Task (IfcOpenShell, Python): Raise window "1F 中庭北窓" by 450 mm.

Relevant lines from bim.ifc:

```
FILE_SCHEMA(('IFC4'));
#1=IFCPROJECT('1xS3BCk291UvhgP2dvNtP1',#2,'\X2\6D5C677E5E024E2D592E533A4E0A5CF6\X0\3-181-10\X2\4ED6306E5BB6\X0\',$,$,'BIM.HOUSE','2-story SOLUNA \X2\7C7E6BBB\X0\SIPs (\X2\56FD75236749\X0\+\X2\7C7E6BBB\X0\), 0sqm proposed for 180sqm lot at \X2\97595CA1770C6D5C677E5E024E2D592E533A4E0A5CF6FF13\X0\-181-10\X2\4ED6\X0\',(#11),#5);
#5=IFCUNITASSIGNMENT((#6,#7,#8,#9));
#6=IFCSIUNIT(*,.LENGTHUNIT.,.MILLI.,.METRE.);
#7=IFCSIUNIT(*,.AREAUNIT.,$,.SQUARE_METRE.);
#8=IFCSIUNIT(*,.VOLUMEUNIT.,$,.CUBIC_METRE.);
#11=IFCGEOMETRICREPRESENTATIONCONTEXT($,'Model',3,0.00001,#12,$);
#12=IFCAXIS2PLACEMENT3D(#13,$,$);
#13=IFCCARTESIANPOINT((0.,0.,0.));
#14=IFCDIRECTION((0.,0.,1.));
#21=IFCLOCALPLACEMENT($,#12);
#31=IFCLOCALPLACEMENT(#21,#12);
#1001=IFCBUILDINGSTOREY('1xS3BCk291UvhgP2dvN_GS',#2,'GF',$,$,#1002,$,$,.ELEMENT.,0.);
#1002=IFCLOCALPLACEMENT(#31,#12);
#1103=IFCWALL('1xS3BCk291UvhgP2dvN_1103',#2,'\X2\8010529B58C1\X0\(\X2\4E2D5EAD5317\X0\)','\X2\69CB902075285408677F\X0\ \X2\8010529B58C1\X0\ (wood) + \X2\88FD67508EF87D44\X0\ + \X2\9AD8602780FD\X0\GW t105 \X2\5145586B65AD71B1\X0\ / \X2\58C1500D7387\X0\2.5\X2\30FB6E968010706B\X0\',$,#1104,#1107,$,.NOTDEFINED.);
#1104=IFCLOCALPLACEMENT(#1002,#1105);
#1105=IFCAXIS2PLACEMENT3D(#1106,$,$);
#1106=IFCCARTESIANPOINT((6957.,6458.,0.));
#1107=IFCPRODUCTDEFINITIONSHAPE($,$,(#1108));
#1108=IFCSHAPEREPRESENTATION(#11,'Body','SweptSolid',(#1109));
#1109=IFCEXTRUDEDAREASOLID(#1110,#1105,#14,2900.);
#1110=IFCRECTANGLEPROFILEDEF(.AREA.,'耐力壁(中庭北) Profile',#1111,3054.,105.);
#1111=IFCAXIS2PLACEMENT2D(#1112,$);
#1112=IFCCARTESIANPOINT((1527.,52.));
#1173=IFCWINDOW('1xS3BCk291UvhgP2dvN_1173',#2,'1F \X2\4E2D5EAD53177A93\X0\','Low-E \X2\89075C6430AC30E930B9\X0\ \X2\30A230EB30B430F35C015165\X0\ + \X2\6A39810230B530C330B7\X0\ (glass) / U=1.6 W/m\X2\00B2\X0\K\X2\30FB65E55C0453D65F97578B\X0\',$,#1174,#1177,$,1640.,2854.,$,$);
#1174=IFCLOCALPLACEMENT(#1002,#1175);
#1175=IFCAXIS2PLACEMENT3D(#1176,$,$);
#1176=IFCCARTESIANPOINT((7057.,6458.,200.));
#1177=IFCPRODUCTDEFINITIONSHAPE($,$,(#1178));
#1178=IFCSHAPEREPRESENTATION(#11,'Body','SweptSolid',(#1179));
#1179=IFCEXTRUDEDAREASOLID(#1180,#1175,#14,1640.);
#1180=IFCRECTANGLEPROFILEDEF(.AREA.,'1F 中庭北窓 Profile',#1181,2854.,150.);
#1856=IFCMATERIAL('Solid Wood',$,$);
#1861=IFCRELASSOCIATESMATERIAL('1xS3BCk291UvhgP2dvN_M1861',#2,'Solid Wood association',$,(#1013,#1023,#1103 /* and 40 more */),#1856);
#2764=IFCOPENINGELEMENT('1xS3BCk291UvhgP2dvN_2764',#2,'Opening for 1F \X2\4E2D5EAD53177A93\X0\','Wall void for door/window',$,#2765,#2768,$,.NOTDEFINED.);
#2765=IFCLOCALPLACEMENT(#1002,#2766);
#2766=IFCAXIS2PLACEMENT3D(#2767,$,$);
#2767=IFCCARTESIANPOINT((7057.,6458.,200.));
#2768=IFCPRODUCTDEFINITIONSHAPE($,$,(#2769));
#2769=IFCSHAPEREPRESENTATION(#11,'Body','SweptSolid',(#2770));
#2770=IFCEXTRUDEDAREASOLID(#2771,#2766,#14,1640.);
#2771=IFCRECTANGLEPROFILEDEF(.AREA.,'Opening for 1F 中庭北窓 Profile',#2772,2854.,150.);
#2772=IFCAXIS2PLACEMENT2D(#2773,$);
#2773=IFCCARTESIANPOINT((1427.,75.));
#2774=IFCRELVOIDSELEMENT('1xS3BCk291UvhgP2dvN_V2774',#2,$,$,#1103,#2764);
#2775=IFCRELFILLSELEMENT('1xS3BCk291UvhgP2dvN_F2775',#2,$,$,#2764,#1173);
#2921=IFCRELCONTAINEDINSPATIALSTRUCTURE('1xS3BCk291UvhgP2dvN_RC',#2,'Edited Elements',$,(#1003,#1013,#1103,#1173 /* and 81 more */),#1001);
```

```python
import numpy as np
import ifcopenshell
import ifcopenshell.api.geometry
import ifcopenshell.util.placement
import ifcopenshell.util.unit

model = ifcopenshell.open("bim.ifc")
unit_scale = ifcopenshell.util.unit.calculate_unit_scale(model)

window = model.by_id(1173)
opening = window.FillsVoids[0].RelatingOpeningElement
dz = 450.0

shift = np.array([0.0, 0.0, dz])
# The window is not placed relative to its opening, so move both.
for product in (opening, window):
    matrix = ifcopenshell.util.placement.get_local_placement(product.ObjectPlacement)
    matrix[:3, 3] += shift
    ifcopenshell.api.geometry.edit_object_placement(model, product=product, matrix=matrix, is_si=False)

print(f"moved by {dz * unit_scale:+.3f} m")

model.write("bim_v2.ifc")
```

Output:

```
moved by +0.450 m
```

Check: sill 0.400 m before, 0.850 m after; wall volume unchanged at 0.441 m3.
